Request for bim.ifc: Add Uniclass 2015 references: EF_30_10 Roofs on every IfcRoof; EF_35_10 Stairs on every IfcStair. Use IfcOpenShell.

First a look at what the model holds.

```python
import ifcopenshell

model = ifcopenshell.open("bim.ifc")
print(model.schema)
print("classifications:", [c.Name for c in model.by_type("IfcClassification")])
for ifc_class in ("IfcDoor", "IfcRoof", "IfcStair", "IfcWall", "IfcWindow"):
    print(ifc_class, len(model.by_type(ifc_class)))
```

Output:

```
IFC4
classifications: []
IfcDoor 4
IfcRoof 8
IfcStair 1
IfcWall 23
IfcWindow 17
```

```python
import ifcopenshell
import ifcopenshell.api.classification

model = ifcopenshell.open("bim.ifc")

system = ifcopenshell.api.classification.add_classification(model, classification="Uniclass 2015")

codes = {
    "IfcRoof": ("EF_30_10", "Roofs"),
    "IfcStair": ("EF_35_10", "Stairs"),
}
for ifc_class, (code, name) in codes.items():
    products = model.by_type(ifc_class)
    ifcopenshell.api.classification.add_reference(
        model, products=products, classification=system, identification=code, name=name
    )
    print(code, len(products))

model.write("bim_rev.ifc")
```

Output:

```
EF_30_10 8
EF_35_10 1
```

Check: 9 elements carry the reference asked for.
